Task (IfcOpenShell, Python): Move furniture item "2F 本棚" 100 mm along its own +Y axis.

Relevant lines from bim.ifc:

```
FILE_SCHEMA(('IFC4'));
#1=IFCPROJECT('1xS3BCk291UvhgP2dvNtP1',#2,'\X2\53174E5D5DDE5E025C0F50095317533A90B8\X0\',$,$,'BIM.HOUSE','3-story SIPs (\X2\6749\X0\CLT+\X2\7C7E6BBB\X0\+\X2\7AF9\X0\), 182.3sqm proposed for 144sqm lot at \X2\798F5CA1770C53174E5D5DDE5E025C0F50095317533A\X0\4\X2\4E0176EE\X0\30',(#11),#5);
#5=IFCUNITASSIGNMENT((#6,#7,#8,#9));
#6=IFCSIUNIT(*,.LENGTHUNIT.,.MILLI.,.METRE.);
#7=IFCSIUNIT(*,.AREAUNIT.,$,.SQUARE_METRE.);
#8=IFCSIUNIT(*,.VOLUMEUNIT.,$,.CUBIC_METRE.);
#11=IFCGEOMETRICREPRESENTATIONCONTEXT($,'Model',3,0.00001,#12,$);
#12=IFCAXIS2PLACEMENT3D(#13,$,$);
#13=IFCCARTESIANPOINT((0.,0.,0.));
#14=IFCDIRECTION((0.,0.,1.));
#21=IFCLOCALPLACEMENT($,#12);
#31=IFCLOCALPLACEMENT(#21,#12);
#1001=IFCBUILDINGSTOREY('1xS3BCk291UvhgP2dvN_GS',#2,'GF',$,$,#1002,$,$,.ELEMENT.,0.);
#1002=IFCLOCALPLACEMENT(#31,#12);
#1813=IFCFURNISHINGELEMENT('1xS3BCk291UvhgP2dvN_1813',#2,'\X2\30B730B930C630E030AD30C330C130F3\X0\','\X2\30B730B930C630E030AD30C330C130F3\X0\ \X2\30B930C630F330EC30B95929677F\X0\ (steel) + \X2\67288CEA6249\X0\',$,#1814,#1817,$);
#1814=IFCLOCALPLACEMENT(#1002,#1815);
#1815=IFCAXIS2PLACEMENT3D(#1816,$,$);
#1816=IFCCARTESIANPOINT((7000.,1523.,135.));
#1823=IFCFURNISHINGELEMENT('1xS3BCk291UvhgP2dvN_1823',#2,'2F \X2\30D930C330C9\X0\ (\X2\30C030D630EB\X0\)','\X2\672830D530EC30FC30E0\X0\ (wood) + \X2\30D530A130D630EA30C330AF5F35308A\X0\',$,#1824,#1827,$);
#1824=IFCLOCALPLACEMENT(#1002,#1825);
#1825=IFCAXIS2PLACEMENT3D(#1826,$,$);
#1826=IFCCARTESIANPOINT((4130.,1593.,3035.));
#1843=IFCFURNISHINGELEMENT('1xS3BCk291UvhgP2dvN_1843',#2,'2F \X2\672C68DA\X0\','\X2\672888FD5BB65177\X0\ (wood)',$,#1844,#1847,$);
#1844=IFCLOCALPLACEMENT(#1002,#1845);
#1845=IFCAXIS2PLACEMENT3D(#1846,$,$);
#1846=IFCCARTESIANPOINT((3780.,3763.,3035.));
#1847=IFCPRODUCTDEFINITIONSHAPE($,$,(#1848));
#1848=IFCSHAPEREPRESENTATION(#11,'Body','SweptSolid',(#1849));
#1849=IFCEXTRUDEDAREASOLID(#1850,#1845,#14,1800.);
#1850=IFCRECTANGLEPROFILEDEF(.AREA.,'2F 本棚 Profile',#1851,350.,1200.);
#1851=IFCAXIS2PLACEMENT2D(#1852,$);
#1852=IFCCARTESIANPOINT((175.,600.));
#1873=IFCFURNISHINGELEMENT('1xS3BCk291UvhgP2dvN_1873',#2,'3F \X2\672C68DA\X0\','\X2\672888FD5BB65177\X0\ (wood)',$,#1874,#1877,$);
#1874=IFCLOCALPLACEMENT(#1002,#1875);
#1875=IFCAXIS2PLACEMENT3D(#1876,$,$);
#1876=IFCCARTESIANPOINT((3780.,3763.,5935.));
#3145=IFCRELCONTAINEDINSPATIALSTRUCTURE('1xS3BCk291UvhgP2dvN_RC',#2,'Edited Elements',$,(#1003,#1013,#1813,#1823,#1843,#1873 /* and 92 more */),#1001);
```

```python
import ifcopenshell
import ifcopenshell.api.geometry
import ifcopenshell.util.placement

model = ifcopenshell.open("bim.ifc")

item = model.by_guid("1xS3BCk291UvhgP2dvN_1843")
matrix = ifcopenshell.util.placement.get_local_placement(item.ObjectPlacement)
matrix[:3, 3] += matrix[:3, 1] * 100.0
ifcopenshell.api.geometry.edit_object_placement(model, product=item, matrix=matrix, is_si=False)

print(ifcopenshell.util.placement.get_local_placement(item.ObjectPlacement).round(3) + 0.0)

model.write("bim_v2.ifc")
```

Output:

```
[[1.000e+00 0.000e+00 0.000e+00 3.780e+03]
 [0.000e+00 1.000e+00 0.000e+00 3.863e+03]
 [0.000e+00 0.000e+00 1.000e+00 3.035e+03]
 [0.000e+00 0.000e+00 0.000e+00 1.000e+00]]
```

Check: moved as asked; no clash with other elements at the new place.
